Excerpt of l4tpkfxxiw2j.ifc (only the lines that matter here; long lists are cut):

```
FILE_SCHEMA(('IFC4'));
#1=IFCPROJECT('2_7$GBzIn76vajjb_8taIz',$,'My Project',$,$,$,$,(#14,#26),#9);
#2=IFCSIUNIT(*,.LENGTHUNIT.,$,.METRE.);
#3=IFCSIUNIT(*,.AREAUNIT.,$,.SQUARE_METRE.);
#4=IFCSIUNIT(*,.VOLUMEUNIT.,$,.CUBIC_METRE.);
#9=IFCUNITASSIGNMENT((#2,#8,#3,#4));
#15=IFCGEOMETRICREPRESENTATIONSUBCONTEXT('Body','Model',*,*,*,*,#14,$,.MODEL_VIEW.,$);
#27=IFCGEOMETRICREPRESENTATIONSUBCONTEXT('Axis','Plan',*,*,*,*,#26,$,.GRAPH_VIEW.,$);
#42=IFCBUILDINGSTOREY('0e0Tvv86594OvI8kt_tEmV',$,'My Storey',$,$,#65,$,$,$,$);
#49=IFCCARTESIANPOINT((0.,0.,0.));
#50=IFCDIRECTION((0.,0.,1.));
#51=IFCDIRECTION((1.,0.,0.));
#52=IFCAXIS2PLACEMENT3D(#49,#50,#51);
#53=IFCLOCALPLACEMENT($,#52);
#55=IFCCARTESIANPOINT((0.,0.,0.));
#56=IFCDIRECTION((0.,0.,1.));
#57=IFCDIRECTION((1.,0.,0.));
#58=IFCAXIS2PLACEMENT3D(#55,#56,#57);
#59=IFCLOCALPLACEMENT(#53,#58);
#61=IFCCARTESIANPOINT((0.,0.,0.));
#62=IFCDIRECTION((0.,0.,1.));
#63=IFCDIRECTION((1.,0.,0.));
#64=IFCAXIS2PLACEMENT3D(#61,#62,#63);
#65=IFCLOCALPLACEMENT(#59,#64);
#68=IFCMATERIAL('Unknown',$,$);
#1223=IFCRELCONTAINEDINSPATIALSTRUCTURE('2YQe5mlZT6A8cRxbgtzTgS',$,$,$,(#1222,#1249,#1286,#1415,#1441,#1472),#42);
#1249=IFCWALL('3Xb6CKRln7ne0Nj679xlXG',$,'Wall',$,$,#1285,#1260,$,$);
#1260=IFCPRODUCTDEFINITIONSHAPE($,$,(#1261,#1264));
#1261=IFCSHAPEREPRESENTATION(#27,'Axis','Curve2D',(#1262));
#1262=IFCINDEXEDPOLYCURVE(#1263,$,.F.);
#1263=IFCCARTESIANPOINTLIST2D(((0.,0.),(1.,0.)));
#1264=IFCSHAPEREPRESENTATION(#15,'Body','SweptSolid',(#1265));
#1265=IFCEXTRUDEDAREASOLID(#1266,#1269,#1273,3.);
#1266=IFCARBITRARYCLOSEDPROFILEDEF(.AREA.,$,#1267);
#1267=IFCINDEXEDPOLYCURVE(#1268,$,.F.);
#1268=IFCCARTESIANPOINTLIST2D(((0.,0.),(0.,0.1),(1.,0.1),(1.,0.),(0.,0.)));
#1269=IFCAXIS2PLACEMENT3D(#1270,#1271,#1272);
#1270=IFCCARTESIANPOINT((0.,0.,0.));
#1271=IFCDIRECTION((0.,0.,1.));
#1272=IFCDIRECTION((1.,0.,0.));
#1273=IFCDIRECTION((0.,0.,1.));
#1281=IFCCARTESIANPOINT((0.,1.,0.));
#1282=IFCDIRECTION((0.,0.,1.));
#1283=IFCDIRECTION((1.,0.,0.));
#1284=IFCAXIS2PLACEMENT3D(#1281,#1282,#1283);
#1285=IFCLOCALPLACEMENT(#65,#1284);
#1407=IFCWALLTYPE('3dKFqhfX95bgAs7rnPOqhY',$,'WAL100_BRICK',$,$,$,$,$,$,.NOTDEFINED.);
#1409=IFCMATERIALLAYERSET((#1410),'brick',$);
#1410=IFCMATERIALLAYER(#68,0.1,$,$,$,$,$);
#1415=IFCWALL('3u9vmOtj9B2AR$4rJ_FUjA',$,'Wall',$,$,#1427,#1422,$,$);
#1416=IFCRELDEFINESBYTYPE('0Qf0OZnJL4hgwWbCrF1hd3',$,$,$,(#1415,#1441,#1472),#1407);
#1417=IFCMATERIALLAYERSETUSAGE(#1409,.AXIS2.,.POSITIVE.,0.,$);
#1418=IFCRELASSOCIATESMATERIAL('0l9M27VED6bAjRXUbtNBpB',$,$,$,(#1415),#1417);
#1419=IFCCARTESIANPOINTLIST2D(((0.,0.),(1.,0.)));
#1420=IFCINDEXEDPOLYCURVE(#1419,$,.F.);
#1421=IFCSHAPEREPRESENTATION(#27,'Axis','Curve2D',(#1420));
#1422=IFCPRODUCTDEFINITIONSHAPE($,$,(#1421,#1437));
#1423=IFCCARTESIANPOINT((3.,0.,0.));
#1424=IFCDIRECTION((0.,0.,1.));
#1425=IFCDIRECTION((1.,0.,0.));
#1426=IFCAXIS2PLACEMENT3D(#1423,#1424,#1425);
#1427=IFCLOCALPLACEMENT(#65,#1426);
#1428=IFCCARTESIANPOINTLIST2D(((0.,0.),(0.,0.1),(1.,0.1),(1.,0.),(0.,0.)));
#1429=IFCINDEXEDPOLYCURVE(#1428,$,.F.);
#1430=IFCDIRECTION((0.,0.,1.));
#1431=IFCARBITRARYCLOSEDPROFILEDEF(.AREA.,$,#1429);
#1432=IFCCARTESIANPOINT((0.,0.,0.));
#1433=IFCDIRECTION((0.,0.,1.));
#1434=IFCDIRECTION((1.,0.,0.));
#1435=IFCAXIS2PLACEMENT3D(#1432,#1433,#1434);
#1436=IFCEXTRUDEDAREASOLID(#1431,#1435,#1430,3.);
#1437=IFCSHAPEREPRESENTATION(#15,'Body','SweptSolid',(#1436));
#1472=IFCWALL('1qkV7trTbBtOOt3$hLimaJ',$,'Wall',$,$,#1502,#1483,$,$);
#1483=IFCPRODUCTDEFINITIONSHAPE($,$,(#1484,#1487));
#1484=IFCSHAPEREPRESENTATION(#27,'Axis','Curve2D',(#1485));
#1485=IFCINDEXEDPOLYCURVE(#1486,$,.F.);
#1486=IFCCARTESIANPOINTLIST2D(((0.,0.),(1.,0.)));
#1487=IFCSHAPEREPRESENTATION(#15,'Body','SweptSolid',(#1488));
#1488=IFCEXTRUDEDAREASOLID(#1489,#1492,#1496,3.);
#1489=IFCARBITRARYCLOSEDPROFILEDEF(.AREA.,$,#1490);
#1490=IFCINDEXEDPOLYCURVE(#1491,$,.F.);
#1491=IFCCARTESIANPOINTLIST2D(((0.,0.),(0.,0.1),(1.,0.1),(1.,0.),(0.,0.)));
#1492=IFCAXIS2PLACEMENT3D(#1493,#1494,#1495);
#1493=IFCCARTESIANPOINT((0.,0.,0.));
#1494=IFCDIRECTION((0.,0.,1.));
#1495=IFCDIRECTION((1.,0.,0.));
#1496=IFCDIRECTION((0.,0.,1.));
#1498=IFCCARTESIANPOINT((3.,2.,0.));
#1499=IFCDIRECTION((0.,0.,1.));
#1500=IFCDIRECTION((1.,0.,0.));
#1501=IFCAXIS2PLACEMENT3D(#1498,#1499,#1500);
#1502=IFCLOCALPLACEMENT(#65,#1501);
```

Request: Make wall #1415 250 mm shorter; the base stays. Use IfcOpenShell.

```python
import ifcopenshell
import ifcopenshell.geom
import ifcopenshell.util.representation
import ifcopenshell.util.shape
import ifcopenshell.util.unit

model = ifcopenshell.open("l4tpkfxxiw2j.ifc")
unit_scale = ifcopenshell.util.unit.calculate_unit_scale(model)
settings = ifcopenshell.geom.settings()


def volume(element):
    """Net volume in cubic metres, openings subtracted."""
    shape = ifcopenshell.geom.create_shape(settings, element)
    return ifcopenshell.util.shape.get_volume(shape.geometry)


wall = model.by_guid("3u9vmOtj9B2AR$4rJ_FUjA")
before = volume(wall)

body = ifcopenshell.util.representation.get_representation(wall, "Model", "Body")
solid = body.Items[0]
old_height = solid.Depth
solid.Depth -= 0.25 / unit_scale
after = volume(wall)

print(f"height {old_height:g} -> {solid.Depth:g}, volume {before:.3f} -> {after:.3f} m3")

model.write("l4tpkfxxiw2j-out.ifc")
```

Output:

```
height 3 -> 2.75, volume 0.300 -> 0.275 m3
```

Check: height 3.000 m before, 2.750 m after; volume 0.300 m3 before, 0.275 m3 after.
